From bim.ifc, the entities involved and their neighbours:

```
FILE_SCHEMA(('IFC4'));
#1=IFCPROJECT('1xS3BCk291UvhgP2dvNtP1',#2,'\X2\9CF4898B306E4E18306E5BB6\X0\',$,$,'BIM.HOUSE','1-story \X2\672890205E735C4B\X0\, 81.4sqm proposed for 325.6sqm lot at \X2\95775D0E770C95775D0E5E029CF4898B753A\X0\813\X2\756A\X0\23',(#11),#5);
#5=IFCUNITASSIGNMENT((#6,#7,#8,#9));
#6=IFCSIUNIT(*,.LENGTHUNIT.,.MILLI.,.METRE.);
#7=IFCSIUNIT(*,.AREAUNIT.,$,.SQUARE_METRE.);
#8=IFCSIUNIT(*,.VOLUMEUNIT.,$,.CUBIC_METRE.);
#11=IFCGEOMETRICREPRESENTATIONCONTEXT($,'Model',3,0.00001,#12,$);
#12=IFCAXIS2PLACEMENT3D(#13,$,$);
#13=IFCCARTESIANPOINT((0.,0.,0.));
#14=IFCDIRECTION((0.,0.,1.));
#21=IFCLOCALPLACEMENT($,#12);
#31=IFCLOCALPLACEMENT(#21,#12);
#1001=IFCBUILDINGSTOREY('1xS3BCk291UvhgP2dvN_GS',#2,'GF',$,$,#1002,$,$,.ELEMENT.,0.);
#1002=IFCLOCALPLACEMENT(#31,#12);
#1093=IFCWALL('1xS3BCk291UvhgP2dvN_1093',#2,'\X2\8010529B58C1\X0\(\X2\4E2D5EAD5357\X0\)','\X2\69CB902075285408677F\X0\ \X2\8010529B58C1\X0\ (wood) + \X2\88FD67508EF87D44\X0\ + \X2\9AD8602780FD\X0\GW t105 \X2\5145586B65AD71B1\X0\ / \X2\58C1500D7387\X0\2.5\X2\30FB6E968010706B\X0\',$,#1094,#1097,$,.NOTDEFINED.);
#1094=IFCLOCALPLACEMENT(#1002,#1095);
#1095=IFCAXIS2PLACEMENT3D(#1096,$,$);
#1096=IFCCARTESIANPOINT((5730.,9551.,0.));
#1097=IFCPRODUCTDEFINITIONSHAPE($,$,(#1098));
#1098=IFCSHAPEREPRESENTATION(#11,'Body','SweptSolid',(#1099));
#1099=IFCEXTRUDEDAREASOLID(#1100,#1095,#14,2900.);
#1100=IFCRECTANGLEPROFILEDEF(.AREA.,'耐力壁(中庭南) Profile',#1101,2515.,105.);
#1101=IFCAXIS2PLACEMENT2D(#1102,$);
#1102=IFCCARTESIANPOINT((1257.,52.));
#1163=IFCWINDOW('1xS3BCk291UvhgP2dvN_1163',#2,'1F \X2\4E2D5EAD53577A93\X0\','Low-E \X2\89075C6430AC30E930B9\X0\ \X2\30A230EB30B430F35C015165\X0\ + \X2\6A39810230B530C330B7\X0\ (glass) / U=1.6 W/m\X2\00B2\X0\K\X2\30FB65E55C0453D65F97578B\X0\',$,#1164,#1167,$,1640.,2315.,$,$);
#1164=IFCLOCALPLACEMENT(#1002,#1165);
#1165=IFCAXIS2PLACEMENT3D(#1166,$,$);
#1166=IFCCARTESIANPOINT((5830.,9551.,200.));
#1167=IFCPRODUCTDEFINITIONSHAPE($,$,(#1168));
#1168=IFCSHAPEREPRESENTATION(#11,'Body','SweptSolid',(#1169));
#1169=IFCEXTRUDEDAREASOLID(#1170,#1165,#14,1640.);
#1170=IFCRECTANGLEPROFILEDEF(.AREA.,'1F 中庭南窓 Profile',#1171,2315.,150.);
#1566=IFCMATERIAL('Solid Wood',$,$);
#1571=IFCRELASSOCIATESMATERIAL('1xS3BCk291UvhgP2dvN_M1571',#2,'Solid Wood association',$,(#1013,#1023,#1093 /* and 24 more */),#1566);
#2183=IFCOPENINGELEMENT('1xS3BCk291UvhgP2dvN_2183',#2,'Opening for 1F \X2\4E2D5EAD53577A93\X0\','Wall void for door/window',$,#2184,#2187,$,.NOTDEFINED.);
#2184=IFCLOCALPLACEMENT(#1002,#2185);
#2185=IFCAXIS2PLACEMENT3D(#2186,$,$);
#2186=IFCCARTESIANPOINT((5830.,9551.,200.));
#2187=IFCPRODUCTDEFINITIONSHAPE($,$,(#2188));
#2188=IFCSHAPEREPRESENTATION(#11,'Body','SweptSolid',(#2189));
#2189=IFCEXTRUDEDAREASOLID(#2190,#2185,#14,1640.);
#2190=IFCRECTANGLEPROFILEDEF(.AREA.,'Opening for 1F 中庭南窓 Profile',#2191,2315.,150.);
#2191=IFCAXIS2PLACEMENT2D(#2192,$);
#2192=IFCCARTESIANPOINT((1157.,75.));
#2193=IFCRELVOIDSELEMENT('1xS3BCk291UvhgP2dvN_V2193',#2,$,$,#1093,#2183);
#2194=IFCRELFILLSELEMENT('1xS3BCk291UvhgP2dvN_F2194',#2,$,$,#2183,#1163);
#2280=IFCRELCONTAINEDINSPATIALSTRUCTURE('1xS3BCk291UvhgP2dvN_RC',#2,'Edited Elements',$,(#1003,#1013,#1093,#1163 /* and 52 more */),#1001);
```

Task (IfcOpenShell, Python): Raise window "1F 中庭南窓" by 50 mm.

```python
import numpy as np
import ifcopenshell
import ifcopenshell.api.geometry
import ifcopenshell.util.placement
import ifcopenshell.util.unit

model = ifcopenshell.open("bim.ifc")
unit_scale = ifcopenshell.util.unit.calculate_unit_scale(model)

window = model.by_guid("1xS3BCk291UvhgP2dvN_1163")
opening = window.FillsVoids[0].RelatingOpeningElement
dz = 50.0

shift = np.array([0.0, 0.0, dz])
# The window is not placed relative to its opening, so move both.
for product in (opening, window):
    matrix = ifcopenshell.util.placement.get_local_placement(product.ObjectPlacement)
    matrix[:3, 3] += shift
    ifcopenshell.api.geometry.edit_object_placement(model, product=product, matrix=matrix, is_si=False)

print(f"moved by {dz * unit_scale:+.3f} m")

model.write("bim_updated.ifc")
```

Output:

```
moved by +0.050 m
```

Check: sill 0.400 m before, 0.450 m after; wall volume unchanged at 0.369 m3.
